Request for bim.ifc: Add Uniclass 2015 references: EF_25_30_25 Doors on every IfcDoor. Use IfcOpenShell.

First a look at what the model holds.

```python
import ifcopenshell

model = ifcopenshell.open("bim.ifc")
print(model.schema)
print("classifications:", [c.Name for c in model.by_type("IfcClassification")])
for ifc_class in ("IfcDoor", "IfcRoof", "IfcStair", "IfcWall", "IfcWindow"):
    print(ifc_class, len(model.by_type(ifc_class)))
```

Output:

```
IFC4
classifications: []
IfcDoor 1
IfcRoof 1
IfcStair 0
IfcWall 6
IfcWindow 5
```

```python
import ifcopenshell
import ifcopenshell.api.classification

model = ifcopenshell.open("bim.ifc")

system = ifcopenshell.api.classification.add_classification(model, classification="Uniclass 2015")

codes = {
    "IfcDoor": ("EF_25_30_25", "Doors"),
}
for ifc_class, (code, name) in codes.items():
    products = model.by_type(ifc_class)
    ifcopenshell.api.classification.add_reference(
        model, products=products, classification=system, identification=code, name=name
    )
    print(code, len(products))

model.write("bim_rev.ifc")
```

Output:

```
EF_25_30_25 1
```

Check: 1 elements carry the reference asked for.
